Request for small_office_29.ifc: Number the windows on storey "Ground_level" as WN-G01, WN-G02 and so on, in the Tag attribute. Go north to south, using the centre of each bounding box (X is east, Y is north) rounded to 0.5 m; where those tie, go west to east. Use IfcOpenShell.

First a look at what the model holds.

```python
import ifcopenshell
import ifcopenshell.util.element
import ifcopenshell.util.placement

model = ifcopenshell.open("small_office_29.ifc")
print(model.schema)
storey = next(s for s in model.by_type("IfcBuildingStorey") if s.Name == "Ground_level")
windows = [e for e in ifcopenshell.util.element.get_decomposition(storey) if e.is_a("IfcWindow")]
for e in sorted(windows, key=lambda e: e.id()):
    origin = ifcopenshell.util.placement.get_local_placement(e.ObjectPlacement)[:3, 3]
    print(e.id(), e.Tag, e.Name, origin.round(2) + 0.0, sep=" | ")
```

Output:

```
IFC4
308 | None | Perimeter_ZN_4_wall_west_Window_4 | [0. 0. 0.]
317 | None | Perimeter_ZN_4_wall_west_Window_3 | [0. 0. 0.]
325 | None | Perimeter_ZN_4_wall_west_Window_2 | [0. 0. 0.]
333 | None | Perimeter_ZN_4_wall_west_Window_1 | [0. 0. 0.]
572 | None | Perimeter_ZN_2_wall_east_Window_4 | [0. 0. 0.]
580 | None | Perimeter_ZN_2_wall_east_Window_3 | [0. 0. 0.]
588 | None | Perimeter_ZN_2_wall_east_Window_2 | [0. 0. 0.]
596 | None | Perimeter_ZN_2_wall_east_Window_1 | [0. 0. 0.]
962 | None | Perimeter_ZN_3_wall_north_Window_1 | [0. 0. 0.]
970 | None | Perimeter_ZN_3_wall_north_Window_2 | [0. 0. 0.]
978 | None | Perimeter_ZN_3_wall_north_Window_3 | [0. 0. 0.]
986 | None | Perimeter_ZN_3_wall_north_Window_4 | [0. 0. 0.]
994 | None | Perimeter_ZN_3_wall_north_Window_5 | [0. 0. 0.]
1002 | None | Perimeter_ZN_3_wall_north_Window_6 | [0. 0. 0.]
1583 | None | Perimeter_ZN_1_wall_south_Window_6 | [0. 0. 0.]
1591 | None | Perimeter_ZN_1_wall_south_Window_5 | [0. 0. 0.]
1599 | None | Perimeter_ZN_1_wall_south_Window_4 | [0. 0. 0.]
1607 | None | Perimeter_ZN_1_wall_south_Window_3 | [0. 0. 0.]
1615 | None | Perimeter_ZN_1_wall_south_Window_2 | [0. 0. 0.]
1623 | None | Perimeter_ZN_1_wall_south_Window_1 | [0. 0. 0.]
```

```python
import ifcopenshell
import ifcopenshell.geom
import ifcopenshell.util.element
import ifcopenshell.util.shape

model = ifcopenshell.open("small_office_29.ifc")
settings = ifcopenshell.geom.settings()
settings.set("use-world-coords", True)


def centre(element):
    shape = ifcopenshell.geom.create_shape(settings, element)
    return ifcopenshell.util.shape.get_bbox_centroid(shape.geometry)


storey = next(s for s in model.by_type("IfcBuildingStorey") if s.Name == "Ground_level")
windows = [e for e in ifcopenshell.util.element.get_decomposition(storey) if e.is_a("IfcWindow")]

# Insertion points can sit at a corner or the storey origin, so sort by the geometry (in metres).
centres = {e: centre(e) for e in windows}
windows.sort(key=lambda e: (-round(centres[e][1] / 0.5), centres[e][0]))

for i, e in enumerate(windows, start=1):
    number = f"WN-G{i:02d}"
    e.Tag = number
    print(e.id(), number)

model.write("small_office_29_rev.ifc")
```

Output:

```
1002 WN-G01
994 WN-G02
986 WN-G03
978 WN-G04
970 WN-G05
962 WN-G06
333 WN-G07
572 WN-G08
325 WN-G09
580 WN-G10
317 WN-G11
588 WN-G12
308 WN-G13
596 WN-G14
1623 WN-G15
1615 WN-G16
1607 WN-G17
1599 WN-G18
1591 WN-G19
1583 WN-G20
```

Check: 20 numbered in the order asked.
